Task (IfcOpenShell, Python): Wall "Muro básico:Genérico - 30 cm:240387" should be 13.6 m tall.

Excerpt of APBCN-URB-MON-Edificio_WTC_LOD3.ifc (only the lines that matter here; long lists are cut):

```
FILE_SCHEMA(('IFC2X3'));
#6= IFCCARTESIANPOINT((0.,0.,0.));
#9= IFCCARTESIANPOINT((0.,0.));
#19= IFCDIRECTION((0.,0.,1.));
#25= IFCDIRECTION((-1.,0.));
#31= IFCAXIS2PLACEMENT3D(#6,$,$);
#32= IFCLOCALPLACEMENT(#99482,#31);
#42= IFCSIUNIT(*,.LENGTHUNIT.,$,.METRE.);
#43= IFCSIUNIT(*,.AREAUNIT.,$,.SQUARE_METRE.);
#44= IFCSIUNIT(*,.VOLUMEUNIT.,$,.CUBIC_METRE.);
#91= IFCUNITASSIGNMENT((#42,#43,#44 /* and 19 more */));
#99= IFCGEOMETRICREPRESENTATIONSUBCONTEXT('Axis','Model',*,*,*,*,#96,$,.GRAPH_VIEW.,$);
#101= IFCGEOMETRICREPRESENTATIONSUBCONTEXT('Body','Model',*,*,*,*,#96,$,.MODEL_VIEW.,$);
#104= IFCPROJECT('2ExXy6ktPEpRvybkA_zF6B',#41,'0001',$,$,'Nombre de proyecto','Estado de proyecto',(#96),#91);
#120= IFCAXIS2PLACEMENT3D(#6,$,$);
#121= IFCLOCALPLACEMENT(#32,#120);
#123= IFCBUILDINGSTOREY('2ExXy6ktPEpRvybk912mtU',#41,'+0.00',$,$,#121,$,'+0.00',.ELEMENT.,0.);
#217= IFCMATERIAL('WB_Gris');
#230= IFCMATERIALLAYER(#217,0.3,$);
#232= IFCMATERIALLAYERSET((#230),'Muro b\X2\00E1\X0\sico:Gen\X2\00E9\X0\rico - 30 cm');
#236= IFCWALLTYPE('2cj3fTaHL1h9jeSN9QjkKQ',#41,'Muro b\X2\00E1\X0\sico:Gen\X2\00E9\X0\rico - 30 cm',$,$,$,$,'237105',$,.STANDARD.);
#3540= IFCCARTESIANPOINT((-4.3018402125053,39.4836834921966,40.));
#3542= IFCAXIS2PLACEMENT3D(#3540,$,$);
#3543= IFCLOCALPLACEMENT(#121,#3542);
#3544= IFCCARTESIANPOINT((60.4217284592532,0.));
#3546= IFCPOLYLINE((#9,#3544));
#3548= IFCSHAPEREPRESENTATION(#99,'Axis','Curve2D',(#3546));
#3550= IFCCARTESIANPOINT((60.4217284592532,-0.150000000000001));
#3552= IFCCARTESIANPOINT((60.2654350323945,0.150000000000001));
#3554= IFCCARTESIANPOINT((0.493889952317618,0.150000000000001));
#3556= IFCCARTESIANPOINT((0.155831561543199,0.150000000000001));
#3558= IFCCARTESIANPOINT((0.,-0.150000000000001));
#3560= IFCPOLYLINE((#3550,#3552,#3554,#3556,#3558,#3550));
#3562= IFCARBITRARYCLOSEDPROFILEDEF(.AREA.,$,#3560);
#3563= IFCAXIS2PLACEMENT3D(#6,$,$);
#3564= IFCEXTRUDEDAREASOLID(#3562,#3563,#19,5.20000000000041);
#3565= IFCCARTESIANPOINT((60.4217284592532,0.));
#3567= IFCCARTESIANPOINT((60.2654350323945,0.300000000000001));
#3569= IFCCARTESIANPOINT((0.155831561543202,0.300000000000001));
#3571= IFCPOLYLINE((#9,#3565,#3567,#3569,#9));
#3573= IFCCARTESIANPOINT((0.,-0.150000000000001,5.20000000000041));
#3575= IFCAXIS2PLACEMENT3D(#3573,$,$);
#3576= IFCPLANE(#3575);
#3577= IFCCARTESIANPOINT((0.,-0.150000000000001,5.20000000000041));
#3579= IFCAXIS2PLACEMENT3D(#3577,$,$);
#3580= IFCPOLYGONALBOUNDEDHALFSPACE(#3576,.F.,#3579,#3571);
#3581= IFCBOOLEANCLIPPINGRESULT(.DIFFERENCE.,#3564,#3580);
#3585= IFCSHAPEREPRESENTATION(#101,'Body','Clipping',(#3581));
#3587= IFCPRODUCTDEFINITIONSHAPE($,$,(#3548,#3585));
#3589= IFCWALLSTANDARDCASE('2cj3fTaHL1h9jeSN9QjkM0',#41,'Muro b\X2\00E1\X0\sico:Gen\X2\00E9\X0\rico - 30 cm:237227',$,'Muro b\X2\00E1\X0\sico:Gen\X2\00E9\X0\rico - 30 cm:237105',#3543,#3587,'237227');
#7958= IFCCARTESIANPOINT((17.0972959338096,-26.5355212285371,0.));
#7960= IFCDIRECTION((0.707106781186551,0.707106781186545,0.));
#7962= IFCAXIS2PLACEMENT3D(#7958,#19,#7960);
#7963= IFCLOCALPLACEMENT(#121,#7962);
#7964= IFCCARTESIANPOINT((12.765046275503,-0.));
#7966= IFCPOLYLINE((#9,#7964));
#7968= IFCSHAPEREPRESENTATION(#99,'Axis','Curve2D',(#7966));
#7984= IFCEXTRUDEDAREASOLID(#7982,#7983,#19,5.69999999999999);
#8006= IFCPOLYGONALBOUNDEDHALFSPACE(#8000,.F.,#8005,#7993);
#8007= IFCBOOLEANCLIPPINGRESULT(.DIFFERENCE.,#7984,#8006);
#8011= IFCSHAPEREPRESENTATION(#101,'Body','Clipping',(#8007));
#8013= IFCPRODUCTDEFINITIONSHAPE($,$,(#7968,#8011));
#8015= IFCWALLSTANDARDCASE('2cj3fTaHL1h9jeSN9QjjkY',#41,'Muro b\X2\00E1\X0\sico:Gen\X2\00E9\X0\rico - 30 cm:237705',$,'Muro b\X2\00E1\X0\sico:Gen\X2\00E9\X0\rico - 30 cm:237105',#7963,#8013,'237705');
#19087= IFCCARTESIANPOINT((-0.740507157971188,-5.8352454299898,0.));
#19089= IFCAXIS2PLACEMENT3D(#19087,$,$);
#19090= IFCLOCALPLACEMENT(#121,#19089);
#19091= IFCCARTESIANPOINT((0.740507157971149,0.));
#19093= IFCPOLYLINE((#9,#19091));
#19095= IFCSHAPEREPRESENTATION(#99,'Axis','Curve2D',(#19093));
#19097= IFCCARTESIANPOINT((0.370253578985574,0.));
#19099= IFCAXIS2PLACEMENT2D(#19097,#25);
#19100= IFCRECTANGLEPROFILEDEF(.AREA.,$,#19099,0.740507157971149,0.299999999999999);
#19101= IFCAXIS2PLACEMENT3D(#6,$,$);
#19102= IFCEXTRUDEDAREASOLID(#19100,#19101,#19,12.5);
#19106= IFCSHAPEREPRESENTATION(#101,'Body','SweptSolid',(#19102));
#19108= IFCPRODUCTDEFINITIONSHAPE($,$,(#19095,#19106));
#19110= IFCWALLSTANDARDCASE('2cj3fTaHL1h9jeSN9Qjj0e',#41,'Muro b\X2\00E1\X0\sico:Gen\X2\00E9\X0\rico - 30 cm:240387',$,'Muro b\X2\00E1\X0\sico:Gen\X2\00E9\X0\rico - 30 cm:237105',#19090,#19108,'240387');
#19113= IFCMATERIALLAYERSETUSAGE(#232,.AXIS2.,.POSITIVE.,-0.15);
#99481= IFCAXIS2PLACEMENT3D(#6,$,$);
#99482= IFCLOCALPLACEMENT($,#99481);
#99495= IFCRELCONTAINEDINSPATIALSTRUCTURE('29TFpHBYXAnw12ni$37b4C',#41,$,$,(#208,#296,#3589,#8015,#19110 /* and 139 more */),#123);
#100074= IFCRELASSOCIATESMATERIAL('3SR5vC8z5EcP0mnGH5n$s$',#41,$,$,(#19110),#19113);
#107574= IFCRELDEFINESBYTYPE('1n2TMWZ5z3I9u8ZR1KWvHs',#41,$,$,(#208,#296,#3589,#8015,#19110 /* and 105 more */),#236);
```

```python
import ifcopenshell
import ifcopenshell.geom
import ifcopenshell.util.representation
import ifcopenshell.util.shape
import ifcopenshell.util.unit

model = ifcopenshell.open("APBCN-URB-MON-Edificio_WTC_LOD3.ifc")
unit_scale = ifcopenshell.util.unit.calculate_unit_scale(model)
settings = ifcopenshell.geom.settings()


def volume(element):
    """Net volume in cubic metres, openings subtracted."""
    shape = ifcopenshell.geom.create_shape(settings, element)
    return ifcopenshell.util.shape.get_volume(shape.geometry)


wall = model.by_guid("2cj3fTaHL1h9jeSN9Qjj0e")
before = volume(wall)

body = ifcopenshell.util.representation.get_representation(wall, "Model", "Body")
solid = body.Items[0]
old_height = solid.Depth
solid.Depth = 13.6 / unit_scale
after = volume(wall)

print(f"height {old_height:g} -> {solid.Depth:g}, volume {before:.3f} -> {after:.3f} m3")

model.write("APBCN-URB-MON-Edificio_WTC_LOD3_updated.ifc")
```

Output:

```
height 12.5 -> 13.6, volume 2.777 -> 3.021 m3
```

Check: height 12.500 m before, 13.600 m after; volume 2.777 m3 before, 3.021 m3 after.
